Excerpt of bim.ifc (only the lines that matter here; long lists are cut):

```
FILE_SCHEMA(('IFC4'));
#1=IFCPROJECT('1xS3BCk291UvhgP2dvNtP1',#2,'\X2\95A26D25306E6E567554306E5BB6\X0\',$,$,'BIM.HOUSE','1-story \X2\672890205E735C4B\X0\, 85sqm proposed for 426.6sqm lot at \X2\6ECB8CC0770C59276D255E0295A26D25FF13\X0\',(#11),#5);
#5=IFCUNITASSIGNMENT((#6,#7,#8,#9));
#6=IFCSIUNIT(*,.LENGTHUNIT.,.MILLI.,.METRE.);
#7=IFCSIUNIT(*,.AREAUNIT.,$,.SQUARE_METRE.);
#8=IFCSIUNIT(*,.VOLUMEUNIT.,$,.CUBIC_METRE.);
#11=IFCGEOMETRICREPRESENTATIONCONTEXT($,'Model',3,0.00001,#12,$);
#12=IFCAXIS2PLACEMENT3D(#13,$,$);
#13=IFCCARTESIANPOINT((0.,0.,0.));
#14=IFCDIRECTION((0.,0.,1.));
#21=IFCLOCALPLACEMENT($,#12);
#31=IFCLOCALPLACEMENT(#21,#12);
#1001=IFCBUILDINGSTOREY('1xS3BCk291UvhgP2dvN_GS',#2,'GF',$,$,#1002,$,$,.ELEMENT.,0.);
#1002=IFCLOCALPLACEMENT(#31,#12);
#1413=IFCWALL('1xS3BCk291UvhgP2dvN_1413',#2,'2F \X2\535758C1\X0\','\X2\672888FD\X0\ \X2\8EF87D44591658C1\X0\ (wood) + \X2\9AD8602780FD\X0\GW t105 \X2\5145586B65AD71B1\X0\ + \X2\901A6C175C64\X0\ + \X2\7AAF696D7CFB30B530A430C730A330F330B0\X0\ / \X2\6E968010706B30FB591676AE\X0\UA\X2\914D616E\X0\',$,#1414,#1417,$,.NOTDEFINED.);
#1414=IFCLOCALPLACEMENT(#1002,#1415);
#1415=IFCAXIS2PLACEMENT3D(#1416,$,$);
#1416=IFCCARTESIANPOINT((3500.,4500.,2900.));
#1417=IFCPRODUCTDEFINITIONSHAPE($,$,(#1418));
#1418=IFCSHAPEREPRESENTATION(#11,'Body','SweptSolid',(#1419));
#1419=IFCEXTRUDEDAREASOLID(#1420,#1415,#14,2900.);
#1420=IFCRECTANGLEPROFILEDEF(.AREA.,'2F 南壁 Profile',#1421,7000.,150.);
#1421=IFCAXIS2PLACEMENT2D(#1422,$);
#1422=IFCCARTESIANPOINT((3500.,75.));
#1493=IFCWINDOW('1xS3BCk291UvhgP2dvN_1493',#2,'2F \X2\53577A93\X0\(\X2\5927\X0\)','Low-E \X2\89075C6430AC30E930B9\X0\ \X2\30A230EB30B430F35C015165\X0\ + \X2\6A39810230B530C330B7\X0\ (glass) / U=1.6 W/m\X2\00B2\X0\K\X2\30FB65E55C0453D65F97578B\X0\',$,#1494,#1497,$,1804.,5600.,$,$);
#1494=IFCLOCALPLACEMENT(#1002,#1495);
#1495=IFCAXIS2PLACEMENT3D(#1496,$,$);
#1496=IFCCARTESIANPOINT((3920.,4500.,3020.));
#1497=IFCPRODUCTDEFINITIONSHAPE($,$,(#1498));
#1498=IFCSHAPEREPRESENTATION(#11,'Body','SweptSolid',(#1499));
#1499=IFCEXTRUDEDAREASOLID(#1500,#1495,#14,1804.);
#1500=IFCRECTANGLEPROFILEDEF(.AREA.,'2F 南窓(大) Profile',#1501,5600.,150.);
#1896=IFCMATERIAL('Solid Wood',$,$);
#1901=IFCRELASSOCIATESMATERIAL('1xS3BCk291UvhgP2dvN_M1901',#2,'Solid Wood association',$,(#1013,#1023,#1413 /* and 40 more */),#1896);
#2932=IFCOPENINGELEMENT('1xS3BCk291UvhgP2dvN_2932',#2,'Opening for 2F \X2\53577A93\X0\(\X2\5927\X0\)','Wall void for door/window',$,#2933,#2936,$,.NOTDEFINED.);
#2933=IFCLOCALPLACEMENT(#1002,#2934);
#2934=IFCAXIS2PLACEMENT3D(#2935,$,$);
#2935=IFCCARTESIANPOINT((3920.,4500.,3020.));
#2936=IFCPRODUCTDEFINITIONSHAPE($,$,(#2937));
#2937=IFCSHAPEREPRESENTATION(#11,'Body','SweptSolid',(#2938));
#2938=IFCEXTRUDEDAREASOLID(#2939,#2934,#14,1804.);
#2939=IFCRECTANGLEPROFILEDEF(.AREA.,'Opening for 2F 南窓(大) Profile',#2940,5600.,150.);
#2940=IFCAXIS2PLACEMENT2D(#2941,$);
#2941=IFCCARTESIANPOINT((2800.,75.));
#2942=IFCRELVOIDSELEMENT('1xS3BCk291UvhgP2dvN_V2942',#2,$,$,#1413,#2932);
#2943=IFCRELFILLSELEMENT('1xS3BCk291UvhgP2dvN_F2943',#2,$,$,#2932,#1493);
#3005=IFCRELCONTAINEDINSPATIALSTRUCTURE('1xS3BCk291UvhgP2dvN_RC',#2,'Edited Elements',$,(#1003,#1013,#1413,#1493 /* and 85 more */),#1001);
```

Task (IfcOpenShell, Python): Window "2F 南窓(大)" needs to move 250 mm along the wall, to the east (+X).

```python
import ifcopenshell
import ifcopenshell.api.geometry
import ifcopenshell.util.placement
import ifcopenshell.util.unit

model = ifcopenshell.open("bim.ifc")
unit_scale = ifcopenshell.util.unit.calculate_unit_scale(model)

window = model.by_guid("1xS3BCk291UvhgP2dvN_1493")
opening = window.FillsVoids[0].RelatingOpeningElement
wall = opening.VoidsElements[0].RelatingBuildingElement

wall_matrix = ifcopenshell.util.placement.get_local_placement(wall.ObjectPlacement)
shift = wall_matrix[:3, 0] * 0.25 / unit_scale
before = ifcopenshell.util.placement.get_local_placement(window.ObjectPlacement)[:3, 3].copy()

# The window is not placed relative to its opening, so move both.
for product in (opening, window):
    matrix = ifcopenshell.util.placement.get_local_placement(product.ObjectPlacement)
    matrix[:3, 3] += shift
    ifcopenshell.api.geometry.edit_object_placement(model, product=product, matrix=matrix, is_si=False)

after = ifcopenshell.util.placement.get_local_placement(window.ObjectPlacement)[:3, 3]
print("window moved by", (after - before).round(3) + 0.0)

model.write("bim_v2.ifc")
```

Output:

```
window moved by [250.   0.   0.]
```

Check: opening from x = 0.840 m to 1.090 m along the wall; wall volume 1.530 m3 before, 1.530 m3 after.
